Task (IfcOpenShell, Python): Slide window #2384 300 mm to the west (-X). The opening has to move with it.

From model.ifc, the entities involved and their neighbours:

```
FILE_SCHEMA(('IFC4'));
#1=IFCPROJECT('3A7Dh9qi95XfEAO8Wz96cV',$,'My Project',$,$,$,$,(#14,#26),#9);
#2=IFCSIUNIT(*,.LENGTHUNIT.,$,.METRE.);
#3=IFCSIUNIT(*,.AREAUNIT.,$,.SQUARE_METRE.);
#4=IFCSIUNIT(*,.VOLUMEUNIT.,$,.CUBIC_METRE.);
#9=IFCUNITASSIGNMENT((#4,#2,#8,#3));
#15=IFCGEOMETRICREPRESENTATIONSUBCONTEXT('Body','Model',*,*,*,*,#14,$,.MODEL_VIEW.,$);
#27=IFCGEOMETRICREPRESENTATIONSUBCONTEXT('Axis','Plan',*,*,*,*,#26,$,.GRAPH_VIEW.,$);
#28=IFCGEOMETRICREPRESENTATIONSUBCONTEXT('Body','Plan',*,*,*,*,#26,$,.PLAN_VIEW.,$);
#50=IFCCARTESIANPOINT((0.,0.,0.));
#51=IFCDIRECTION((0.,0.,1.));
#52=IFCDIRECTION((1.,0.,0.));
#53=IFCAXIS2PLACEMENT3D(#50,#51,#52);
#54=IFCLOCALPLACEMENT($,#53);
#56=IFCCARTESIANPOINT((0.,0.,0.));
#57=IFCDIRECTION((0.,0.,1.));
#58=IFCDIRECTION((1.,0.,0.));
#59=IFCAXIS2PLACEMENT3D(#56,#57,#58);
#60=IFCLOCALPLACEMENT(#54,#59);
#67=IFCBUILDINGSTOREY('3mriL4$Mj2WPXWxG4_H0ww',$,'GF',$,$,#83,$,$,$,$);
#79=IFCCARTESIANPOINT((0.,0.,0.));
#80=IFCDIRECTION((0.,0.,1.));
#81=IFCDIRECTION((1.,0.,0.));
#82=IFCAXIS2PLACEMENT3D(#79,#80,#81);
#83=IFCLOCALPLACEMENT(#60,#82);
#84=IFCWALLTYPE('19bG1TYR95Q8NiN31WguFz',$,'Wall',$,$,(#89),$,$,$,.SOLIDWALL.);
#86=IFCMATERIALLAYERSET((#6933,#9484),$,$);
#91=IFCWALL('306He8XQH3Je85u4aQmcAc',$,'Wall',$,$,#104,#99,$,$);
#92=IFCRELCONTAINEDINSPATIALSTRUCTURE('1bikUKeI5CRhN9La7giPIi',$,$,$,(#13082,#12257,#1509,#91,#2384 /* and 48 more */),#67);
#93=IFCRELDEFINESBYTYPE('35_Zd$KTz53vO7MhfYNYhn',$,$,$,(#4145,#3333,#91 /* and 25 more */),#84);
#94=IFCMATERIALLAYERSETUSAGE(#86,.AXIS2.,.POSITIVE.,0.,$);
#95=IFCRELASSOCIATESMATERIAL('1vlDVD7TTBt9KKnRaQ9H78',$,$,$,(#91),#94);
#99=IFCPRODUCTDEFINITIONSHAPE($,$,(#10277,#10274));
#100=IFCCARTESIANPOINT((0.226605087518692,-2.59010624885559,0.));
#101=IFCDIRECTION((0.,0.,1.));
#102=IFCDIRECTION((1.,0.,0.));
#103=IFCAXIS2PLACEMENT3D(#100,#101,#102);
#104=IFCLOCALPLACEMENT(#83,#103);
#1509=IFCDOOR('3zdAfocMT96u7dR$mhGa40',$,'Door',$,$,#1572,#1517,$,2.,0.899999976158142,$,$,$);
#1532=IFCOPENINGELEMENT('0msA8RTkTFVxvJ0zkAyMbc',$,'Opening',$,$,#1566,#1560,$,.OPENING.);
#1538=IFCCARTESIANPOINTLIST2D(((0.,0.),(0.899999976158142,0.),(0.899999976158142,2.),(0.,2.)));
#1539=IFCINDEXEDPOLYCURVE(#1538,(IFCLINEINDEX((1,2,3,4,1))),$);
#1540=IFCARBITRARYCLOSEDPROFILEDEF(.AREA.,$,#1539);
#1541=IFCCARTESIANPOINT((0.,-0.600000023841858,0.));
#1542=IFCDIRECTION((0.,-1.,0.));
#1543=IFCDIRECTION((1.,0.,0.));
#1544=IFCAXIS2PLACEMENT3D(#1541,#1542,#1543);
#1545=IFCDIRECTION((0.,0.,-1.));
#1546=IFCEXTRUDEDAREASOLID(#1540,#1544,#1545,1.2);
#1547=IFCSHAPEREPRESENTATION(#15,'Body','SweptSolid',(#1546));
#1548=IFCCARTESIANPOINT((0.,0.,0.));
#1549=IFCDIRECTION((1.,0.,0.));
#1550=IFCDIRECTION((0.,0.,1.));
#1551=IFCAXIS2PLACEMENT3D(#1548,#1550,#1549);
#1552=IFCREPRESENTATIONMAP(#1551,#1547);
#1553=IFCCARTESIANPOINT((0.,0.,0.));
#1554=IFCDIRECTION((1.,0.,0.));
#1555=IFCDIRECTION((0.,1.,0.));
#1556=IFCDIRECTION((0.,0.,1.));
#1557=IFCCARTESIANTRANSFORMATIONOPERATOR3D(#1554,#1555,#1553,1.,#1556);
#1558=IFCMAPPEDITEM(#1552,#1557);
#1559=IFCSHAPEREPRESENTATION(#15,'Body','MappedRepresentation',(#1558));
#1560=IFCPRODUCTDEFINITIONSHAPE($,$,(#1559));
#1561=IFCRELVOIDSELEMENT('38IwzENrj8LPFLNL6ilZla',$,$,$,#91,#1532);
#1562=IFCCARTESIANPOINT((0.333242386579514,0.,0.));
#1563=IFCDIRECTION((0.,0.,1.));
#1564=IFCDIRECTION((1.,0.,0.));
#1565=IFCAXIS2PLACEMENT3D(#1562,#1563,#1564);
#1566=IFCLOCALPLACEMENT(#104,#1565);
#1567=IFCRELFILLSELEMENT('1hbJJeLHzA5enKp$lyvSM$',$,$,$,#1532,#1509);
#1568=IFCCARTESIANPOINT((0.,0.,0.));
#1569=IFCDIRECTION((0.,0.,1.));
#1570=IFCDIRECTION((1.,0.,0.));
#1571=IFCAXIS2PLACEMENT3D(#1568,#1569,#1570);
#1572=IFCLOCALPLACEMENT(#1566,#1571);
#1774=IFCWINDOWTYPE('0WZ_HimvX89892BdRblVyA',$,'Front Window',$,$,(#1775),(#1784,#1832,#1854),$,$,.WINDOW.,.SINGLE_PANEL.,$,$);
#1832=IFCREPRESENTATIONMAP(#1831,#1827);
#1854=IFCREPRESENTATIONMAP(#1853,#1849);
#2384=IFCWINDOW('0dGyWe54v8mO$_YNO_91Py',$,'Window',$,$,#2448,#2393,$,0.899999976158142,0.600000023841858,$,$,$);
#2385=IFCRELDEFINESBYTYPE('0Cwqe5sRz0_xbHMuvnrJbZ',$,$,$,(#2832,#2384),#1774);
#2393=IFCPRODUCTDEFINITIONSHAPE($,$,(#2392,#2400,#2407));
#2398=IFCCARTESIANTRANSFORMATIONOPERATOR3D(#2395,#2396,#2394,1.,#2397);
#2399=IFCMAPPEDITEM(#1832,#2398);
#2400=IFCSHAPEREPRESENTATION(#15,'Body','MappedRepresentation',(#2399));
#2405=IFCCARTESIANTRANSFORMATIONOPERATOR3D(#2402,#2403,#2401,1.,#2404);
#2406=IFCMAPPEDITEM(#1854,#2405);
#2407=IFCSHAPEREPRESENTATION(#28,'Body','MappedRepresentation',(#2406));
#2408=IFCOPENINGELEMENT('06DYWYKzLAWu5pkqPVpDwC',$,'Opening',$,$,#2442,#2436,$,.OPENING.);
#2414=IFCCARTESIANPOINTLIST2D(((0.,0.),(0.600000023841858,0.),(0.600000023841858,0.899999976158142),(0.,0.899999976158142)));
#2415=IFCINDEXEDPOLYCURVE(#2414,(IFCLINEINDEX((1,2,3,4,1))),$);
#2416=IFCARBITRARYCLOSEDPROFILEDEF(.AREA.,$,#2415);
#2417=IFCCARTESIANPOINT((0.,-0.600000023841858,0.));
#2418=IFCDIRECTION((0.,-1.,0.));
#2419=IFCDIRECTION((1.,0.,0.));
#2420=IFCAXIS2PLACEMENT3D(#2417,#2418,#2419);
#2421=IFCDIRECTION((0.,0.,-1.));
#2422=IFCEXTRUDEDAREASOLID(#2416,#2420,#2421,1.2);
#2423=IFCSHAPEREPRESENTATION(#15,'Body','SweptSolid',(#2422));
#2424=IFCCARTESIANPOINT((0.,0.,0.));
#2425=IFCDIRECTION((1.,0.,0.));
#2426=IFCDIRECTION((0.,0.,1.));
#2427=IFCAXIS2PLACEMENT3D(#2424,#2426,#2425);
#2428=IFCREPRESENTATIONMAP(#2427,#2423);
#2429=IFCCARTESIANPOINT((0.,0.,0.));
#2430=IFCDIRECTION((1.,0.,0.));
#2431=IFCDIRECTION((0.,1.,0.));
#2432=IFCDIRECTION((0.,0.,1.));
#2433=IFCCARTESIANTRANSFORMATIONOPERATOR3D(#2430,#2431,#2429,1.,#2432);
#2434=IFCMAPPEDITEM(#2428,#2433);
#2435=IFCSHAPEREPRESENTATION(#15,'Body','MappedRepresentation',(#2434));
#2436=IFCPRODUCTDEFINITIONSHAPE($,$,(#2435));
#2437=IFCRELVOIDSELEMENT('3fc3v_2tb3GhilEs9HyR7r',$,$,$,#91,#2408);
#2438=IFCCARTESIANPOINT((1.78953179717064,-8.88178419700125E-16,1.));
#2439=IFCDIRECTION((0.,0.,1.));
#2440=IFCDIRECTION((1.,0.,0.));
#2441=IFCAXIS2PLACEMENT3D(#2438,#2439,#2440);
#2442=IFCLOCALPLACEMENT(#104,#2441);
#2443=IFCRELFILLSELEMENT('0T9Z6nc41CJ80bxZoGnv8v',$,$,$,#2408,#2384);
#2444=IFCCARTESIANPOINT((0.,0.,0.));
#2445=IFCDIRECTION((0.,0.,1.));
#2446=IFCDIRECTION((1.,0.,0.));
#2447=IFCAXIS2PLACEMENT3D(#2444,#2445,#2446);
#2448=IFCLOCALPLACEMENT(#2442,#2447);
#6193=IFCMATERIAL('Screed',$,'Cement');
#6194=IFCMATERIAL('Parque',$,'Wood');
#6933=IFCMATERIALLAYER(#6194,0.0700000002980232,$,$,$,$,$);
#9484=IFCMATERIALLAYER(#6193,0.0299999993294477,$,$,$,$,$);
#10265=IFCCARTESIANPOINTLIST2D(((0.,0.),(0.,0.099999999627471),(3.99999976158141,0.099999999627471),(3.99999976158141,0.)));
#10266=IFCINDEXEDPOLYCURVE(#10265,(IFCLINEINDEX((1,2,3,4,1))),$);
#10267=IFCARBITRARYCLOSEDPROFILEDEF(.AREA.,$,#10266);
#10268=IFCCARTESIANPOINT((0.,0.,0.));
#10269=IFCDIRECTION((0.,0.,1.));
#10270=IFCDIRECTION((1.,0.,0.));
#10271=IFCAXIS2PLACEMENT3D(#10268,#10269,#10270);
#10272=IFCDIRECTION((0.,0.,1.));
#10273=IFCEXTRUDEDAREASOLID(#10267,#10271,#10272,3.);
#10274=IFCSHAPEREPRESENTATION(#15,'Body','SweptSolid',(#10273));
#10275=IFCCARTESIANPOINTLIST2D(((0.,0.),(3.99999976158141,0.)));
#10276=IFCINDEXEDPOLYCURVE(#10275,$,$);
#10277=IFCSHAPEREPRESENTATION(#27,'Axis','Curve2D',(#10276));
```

```python
import ifcopenshell
import ifcopenshell.api.geometry
import ifcopenshell.util.placement
import ifcopenshell.util.unit

model = ifcopenshell.open("model.ifc")
unit_scale = ifcopenshell.util.unit.calculate_unit_scale(model)

window = model.by_guid("0dGyWe54v8mO$_YNO_91Py")
opening = window.FillsVoids[0].RelatingOpeningElement
wall = opening.VoidsElements[0].RelatingBuildingElement

wall_matrix = ifcopenshell.util.placement.get_local_placement(wall.ObjectPlacement)
shift = wall_matrix[:3, 0] * -0.3 / unit_scale
before = ifcopenshell.util.placement.get_local_placement(window.ObjectPlacement)[:3, 3].copy()

# The window is placed relative to its opening, so it follows when the opening moves.
matrix = ifcopenshell.util.placement.get_local_placement(opening.ObjectPlacement)
matrix[:3, 3] += shift
ifcopenshell.api.geometry.edit_object_placement(
    model, product=opening, matrix=matrix, is_si=False, should_transform_children=True
)

after = ifcopenshell.util.placement.get_local_placement(window.ObjectPlacement)[:3, 3]
print("window moved by", (after - before).round(3) + 0.0)

model.write("model_rev.ifc")
```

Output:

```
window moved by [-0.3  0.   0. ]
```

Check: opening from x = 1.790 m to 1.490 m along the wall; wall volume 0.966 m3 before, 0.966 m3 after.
